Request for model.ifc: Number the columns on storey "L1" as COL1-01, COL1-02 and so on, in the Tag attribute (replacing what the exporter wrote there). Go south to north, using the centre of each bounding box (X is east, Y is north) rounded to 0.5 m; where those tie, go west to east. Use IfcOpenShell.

First a look at what the model holds.

```python
import ifcopenshell
import ifcopenshell.util.element
import ifcopenshell.util.placement

model = ifcopenshell.open("model.ifc")
print(model.schema)
storey = next(s for s in model.by_type("IfcBuildingStorey") if s.Name == "L1")
columns = [e for e in ifcopenshell.util.element.get_decomposition(storey) if e.is_a("IfcColumn")]
for e in sorted(columns, key=lambda e: e.id()):
    origin = ifcopenshell.util.placement.get_local_placement(e.ObjectPlacement)[:3, 3]
    print(e.id(), e.Tag, e.Name, origin.round(2) + 0.0, sep=" | ")
```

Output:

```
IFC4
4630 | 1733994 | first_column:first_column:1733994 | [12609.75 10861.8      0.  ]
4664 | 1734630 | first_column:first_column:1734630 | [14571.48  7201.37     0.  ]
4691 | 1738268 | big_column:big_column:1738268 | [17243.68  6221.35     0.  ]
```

```python
import ifcopenshell
import ifcopenshell.geom
import ifcopenshell.util.element
import ifcopenshell.util.shape

model = ifcopenshell.open("model.ifc")
settings = ifcopenshell.geom.settings()
settings.set("use-world-coords", True)


def centre(element):
    shape = ifcopenshell.geom.create_shape(settings, element)
    return ifcopenshell.util.shape.get_bbox_centroid(shape.geometry)


storey = next(s for s in model.by_type("IfcBuildingStorey") if s.Name == "L1")
columns = [e for e in ifcopenshell.util.element.get_decomposition(storey) if e.is_a("IfcColumn")]

# Insertion points can sit at a corner or the storey origin, so sort by the geometry (in metres).
centres = {e: centre(e) for e in columns}
columns.sort(key=lambda e: (round(centres[e][1] / 0.5), centres[e][0]))

for i, e in enumerate(columns, start=1):
    number = f"COL1-{i:02d}"
    e.Tag = number
    print(e.id(), number)

model.write("model_updated.ifc")
```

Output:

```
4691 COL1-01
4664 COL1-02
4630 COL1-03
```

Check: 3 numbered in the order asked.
